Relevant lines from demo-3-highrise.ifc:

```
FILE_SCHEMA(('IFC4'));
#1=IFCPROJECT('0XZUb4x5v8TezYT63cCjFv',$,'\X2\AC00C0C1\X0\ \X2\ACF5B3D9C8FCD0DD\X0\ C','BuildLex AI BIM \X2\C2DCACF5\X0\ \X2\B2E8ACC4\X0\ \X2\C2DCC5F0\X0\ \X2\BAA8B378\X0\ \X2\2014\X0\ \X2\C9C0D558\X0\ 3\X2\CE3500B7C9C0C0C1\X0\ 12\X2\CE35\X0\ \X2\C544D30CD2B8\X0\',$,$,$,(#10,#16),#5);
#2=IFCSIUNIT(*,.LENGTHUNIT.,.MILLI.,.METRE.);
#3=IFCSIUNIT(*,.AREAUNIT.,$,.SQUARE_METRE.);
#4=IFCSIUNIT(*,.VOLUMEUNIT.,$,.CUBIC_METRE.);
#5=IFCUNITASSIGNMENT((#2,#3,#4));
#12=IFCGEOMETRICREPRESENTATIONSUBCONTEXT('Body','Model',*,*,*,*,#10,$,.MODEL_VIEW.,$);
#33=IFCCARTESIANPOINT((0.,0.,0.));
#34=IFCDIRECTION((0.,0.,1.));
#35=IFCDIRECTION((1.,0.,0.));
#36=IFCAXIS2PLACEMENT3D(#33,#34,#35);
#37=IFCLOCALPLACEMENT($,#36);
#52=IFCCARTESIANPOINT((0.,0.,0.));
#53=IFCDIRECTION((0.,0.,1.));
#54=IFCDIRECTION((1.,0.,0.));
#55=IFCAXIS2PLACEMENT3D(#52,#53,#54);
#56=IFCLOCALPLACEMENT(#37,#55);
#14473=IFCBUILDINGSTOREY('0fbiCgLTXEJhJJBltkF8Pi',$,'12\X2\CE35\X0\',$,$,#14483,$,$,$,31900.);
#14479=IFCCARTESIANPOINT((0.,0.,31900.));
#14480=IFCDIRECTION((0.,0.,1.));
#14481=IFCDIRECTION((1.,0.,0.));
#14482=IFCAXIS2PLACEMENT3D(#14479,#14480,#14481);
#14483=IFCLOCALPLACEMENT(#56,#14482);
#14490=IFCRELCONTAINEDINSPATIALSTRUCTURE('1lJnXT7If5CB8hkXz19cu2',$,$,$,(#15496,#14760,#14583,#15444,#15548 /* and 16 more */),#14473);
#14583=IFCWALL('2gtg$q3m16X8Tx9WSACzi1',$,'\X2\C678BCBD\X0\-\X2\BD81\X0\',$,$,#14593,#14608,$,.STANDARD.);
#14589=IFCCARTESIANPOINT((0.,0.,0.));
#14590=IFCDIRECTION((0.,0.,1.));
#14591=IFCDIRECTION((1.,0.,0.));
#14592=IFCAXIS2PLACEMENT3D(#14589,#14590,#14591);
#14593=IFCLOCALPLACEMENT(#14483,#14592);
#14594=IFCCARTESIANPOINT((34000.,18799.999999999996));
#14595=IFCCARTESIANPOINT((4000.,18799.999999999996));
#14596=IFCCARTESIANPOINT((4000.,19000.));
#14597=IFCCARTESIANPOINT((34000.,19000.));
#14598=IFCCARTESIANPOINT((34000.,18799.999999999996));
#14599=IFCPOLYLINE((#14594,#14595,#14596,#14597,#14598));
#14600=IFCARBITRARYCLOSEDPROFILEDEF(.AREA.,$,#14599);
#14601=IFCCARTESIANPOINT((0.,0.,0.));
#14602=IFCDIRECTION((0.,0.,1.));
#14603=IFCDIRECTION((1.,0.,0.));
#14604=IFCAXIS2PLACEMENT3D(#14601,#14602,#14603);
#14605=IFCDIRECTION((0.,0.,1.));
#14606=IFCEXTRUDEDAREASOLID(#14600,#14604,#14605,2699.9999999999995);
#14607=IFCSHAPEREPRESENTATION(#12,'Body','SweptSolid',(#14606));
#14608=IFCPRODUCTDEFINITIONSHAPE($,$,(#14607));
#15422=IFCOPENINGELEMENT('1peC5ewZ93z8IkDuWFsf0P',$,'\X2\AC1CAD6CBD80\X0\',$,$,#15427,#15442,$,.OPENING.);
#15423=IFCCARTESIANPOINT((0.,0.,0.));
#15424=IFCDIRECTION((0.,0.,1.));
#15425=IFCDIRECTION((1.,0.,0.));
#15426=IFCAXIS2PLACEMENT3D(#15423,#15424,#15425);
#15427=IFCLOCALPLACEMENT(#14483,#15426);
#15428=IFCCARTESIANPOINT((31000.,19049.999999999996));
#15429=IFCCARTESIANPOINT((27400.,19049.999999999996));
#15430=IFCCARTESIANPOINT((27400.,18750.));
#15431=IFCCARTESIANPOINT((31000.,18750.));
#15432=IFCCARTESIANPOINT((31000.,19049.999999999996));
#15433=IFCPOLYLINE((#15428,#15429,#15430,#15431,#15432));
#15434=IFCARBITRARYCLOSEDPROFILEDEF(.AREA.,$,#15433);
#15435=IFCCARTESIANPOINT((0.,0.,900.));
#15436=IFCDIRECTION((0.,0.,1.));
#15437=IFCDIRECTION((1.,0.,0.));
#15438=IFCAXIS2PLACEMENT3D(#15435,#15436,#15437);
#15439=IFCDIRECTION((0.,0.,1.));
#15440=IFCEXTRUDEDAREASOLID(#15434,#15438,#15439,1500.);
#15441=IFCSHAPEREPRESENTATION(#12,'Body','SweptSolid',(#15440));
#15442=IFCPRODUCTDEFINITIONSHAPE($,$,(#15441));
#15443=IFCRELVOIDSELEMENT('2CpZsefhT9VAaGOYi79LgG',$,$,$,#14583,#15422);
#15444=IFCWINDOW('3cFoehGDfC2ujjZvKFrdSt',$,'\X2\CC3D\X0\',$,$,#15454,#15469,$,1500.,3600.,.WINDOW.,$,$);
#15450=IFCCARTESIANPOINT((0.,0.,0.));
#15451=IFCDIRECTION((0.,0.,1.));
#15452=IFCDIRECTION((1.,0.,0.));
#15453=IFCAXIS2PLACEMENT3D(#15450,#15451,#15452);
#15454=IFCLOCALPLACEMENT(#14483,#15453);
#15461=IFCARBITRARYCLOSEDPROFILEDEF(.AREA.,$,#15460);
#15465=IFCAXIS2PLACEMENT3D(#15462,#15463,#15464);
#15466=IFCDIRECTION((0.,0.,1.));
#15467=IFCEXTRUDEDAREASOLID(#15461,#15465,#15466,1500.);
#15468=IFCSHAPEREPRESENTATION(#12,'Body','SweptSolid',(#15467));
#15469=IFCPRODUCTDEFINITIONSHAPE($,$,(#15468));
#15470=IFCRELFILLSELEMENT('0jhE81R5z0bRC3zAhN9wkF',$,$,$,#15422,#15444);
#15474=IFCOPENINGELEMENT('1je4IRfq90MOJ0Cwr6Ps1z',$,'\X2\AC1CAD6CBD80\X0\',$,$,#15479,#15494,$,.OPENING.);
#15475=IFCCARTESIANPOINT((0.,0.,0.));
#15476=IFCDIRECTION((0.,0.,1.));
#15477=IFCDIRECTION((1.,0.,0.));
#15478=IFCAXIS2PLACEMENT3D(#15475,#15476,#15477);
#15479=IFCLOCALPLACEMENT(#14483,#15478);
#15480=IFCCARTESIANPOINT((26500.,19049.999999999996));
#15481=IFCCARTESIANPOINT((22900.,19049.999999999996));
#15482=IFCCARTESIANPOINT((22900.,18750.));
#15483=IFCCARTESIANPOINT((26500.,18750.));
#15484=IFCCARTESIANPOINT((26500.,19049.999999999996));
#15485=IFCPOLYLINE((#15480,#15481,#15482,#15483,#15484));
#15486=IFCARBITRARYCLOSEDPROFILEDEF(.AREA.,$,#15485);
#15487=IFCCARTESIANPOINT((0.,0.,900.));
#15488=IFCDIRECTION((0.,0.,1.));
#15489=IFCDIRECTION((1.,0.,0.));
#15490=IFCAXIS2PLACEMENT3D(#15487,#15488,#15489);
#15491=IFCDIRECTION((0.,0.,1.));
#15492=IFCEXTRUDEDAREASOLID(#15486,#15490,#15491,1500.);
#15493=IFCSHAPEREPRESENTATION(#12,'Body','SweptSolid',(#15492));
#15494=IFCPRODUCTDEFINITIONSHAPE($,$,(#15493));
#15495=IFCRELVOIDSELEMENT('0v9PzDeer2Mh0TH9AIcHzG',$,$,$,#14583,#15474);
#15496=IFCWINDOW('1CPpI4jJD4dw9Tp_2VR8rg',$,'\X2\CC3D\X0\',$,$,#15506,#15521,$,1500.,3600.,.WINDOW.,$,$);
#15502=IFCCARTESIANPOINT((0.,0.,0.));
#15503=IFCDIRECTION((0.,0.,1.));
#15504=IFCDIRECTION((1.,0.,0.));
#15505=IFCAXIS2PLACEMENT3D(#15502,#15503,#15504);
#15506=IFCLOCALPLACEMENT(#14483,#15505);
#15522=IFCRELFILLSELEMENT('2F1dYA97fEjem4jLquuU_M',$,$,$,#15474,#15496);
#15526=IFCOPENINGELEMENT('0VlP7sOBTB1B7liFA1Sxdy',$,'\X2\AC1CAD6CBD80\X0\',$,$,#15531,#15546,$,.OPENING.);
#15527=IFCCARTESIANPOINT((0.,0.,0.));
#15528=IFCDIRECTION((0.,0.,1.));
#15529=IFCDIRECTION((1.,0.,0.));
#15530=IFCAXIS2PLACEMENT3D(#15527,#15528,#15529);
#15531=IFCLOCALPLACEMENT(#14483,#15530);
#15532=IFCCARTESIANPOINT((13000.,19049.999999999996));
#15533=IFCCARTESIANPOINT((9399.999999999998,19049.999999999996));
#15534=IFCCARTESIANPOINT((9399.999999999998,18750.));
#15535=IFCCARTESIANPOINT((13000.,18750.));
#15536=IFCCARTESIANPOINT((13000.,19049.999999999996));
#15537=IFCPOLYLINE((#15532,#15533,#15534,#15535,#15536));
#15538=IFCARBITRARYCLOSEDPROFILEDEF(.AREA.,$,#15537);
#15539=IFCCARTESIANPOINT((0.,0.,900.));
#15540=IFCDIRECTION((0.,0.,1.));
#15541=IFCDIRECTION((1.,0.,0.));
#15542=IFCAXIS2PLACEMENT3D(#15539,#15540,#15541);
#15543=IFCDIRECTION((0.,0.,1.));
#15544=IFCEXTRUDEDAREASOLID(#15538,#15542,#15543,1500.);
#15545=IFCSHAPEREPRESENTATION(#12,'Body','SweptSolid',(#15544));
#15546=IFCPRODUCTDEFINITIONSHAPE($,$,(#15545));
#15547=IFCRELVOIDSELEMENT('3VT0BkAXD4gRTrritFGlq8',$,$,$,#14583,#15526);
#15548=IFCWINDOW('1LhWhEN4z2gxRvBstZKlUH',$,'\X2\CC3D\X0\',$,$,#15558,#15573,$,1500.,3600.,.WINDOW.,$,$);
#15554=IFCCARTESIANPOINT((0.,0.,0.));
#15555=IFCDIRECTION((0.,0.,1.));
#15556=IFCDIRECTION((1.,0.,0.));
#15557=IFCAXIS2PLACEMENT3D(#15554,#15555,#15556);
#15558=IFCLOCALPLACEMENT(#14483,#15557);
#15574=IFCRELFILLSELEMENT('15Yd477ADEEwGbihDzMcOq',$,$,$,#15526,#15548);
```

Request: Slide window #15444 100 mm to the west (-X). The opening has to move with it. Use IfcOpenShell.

```python
import ifcopenshell
import ifcopenshell.api.geometry
import ifcopenshell.util.placement
import ifcopenshell.util.unit

model = ifcopenshell.open("demo-3-highrise.ifc")
unit_scale = ifcopenshell.util.unit.calculate_unit_scale(model)

window = model.by_id(15444)
opening = window.FillsVoids[0].RelatingOpeningElement
wall = opening.VoidsElements[0].RelatingBuildingElement

wall_matrix = ifcopenshell.util.placement.get_local_placement(wall.ObjectPlacement)
shift = wall_matrix[:3, 0] * -0.1 / unit_scale
before = ifcopenshell.util.placement.get_local_placement(window.ObjectPlacement)[:3, 3].copy()

# The window is not placed relative to its opening, so move both.
for product in (opening, window):
    matrix = ifcopenshell.util.placement.get_local_placement(product.ObjectPlacement)
    matrix[:3, 3] += shift
    ifcopenshell.api.geometry.edit_object_placement(model, product=product, matrix=matrix, is_si=False)

after = ifcopenshell.util.placement.get_local_placement(window.ObjectPlacement)[:3, 3]
print("window moved by", (after - before).round(3) + 0.0)

model.write("demo-3-highrise_rev.ifc")
```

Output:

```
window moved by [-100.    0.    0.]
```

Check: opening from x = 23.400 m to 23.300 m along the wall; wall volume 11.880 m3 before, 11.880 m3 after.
